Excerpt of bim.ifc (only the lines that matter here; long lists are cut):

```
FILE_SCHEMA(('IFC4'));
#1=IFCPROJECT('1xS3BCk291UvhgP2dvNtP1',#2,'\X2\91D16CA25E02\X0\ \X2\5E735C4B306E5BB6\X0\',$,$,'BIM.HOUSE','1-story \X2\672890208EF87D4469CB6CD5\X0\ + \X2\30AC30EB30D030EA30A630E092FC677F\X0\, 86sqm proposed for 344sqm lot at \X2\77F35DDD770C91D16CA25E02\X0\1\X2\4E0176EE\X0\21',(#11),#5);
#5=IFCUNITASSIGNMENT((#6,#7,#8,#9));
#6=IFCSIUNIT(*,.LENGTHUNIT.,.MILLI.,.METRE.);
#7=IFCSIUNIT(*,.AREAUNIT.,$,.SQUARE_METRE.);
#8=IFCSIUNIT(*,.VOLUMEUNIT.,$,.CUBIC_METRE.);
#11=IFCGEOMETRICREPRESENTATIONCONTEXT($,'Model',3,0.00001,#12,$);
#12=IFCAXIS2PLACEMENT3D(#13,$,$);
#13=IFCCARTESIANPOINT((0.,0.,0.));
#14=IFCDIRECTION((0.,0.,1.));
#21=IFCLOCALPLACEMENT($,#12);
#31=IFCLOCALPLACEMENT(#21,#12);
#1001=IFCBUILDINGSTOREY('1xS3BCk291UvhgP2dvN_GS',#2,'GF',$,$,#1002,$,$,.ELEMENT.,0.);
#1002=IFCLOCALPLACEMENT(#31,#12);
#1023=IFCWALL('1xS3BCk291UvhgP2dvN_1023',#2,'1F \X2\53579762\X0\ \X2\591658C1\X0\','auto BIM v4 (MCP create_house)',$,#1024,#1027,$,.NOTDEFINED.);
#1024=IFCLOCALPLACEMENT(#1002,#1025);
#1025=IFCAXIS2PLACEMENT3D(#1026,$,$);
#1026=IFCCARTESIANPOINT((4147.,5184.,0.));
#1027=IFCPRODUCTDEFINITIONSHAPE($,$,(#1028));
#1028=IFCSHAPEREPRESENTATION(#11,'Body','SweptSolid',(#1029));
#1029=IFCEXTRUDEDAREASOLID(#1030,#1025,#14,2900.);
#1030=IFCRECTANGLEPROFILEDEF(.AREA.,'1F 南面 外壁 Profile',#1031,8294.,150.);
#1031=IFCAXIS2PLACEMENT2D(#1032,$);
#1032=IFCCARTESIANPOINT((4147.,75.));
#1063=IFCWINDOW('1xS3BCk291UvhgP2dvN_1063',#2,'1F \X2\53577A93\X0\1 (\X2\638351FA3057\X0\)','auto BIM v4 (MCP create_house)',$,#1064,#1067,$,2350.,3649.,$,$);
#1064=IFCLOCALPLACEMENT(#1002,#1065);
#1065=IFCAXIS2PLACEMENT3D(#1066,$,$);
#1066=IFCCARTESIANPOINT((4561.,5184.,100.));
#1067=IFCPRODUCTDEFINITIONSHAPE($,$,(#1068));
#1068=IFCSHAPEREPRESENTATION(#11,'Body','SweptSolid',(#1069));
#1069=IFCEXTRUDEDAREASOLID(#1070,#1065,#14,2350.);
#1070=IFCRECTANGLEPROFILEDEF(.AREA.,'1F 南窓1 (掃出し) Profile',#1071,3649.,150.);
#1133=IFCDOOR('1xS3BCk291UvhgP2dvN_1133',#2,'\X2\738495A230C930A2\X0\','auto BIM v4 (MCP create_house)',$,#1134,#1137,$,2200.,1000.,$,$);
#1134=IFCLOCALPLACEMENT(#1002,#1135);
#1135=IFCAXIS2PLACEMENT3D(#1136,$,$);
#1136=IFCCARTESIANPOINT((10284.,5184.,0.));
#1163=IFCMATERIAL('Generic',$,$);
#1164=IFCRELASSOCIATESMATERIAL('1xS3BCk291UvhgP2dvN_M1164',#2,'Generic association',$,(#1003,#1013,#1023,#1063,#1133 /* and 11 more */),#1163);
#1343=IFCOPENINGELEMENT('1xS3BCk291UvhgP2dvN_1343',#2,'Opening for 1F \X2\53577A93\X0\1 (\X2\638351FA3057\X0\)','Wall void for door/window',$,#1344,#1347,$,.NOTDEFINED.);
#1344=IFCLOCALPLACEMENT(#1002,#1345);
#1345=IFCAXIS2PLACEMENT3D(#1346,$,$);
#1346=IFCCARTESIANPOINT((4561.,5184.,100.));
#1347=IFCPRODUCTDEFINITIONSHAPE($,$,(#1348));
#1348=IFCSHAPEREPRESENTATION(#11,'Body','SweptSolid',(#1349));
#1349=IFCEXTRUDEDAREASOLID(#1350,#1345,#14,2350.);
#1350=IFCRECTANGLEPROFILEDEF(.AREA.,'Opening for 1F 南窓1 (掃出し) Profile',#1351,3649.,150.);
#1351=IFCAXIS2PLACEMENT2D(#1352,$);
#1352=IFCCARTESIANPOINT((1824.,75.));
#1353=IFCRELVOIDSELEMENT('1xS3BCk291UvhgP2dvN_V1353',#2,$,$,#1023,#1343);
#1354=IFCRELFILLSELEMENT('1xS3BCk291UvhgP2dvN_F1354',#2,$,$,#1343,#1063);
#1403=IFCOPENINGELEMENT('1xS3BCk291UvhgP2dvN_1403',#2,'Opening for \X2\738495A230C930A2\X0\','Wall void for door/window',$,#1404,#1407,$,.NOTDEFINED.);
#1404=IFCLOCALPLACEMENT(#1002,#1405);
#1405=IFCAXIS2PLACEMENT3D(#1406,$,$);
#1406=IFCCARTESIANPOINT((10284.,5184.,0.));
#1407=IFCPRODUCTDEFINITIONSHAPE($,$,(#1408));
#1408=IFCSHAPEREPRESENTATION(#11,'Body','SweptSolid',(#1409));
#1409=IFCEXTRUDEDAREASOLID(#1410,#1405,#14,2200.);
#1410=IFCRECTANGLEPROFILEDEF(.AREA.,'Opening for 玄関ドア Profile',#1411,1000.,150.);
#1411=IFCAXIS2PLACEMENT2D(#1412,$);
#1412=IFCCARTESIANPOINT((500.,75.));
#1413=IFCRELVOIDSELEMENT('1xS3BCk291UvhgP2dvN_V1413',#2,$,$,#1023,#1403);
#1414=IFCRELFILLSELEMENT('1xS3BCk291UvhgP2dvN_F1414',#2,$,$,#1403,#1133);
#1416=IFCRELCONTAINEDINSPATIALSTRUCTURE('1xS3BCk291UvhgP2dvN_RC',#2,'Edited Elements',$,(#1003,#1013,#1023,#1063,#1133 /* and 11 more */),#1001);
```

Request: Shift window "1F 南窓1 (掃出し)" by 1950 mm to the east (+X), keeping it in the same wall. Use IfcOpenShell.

```python
import ifcopenshell
import ifcopenshell.api.geometry
import ifcopenshell.util.placement
import ifcopenshell.util.unit

model = ifcopenshell.open("bim.ifc")
unit_scale = ifcopenshell.util.unit.calculate_unit_scale(model)

window = model.by_guid("1xS3BCk291UvhgP2dvN_1063")
opening = window.FillsVoids[0].RelatingOpeningElement
wall = opening.VoidsElements[0].RelatingBuildingElement

wall_matrix = ifcopenshell.util.placement.get_local_placement(wall.ObjectPlacement)
shift = wall_matrix[:3, 0] * 1.95 / unit_scale
before = ifcopenshell.util.placement.get_local_placement(window.ObjectPlacement)[:3, 3].copy()

# The window is not placed relative to its opening, so move both.
for product in (opening, window):
    matrix = ifcopenshell.util.placement.get_local_placement(product.ObjectPlacement)
    matrix[:3, 3] += shift
    ifcopenshell.api.geometry.edit_object_placement(model, product=product, matrix=matrix, is_si=False)

after = ifcopenshell.util.placement.get_local_placement(window.ObjectPlacement)[:3, 3]
print("window moved by", (after - before).round(3) + 0.0)

model.write("bim-out.ifc")
```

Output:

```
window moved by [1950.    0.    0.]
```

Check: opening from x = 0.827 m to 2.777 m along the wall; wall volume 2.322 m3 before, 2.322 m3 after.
